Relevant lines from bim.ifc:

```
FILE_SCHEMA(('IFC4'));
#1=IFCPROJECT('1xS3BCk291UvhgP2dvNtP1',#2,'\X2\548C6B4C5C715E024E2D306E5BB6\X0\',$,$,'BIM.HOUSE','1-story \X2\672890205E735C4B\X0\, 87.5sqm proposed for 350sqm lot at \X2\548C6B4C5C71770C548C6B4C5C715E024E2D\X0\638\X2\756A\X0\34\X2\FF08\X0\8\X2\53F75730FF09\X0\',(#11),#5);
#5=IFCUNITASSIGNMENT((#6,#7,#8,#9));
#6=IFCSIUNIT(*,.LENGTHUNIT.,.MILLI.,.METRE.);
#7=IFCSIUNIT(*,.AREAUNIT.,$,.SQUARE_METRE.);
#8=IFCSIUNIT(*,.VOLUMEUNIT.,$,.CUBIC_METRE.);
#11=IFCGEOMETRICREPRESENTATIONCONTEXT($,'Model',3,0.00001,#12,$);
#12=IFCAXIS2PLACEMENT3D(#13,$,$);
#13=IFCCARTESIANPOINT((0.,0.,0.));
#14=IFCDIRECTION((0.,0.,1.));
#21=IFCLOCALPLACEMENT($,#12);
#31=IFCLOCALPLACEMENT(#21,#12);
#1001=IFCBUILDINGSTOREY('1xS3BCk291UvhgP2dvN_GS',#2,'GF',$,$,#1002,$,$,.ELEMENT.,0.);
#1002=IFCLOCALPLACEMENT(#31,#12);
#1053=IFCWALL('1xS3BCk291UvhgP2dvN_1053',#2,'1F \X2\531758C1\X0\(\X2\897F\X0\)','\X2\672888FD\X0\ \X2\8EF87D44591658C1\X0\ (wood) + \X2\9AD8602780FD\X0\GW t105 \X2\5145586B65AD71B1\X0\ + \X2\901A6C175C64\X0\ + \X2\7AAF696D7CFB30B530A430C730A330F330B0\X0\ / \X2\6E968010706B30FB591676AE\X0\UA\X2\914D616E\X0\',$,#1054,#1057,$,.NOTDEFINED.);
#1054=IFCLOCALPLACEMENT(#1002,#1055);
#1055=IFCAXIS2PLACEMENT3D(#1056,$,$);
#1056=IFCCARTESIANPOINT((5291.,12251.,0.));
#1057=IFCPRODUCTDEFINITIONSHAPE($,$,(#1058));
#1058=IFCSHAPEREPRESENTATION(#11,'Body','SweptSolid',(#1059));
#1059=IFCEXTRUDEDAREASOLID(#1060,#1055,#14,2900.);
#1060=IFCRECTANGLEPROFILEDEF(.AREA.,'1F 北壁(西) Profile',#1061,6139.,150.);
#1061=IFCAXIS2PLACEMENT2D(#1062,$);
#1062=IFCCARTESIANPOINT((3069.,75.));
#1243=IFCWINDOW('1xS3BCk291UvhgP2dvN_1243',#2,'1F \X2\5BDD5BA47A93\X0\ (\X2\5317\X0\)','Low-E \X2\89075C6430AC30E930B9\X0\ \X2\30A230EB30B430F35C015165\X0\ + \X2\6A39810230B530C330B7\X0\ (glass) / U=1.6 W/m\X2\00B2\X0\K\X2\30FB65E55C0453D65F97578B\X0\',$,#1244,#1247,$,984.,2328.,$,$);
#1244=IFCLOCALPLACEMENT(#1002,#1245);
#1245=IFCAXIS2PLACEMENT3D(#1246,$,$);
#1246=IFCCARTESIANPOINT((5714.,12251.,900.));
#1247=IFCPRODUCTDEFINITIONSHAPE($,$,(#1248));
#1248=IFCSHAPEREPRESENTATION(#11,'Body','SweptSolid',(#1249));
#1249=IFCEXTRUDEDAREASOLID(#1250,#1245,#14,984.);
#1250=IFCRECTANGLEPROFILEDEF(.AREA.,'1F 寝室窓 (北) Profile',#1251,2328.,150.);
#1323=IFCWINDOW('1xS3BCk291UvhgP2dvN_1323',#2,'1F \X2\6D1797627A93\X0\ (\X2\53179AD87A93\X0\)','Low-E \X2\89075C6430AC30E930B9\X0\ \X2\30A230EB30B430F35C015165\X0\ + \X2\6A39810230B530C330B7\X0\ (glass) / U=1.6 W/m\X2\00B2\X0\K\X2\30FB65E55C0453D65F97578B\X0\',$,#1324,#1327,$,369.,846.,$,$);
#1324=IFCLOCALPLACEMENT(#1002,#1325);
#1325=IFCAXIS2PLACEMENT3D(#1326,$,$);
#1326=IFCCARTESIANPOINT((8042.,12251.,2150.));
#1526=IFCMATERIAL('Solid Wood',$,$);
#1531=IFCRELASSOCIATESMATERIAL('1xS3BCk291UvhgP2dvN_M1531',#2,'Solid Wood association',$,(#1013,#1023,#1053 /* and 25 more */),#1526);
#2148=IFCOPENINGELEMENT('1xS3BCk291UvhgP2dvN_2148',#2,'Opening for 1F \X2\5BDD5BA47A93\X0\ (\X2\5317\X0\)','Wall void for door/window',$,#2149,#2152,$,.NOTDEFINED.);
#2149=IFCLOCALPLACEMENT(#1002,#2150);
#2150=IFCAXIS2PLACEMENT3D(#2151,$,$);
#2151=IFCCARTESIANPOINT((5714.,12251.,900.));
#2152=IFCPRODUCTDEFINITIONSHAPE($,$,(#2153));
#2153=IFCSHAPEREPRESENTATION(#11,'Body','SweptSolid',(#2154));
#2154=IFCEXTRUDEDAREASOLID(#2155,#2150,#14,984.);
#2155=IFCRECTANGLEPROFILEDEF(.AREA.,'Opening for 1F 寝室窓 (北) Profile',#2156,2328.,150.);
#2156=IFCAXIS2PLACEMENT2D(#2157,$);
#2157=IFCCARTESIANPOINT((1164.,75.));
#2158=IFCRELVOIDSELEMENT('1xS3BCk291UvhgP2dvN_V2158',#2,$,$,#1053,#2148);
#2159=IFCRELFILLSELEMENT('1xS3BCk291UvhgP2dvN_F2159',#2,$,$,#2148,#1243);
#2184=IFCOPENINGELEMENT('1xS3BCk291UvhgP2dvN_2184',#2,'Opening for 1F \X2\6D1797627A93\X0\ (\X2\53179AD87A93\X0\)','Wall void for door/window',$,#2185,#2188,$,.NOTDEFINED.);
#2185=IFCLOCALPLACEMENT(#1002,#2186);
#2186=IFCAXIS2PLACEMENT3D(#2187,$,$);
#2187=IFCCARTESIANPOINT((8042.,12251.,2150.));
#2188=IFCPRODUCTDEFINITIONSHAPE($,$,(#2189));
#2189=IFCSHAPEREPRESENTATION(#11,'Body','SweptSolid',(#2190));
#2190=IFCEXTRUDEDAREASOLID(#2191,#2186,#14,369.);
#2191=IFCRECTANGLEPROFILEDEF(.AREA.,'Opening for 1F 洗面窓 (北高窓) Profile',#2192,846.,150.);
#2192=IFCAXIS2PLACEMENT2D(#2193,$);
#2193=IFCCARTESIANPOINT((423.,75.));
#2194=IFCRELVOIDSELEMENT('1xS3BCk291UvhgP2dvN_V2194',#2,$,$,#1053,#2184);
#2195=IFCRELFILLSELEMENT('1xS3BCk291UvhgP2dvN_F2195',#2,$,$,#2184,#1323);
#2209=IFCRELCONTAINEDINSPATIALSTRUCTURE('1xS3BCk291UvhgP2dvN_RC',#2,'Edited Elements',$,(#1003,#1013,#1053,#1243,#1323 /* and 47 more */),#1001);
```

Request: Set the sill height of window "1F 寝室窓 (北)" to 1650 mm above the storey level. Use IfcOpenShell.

```python
import numpy as np
import ifcopenshell
import ifcopenshell.api.geometry
import ifcopenshell.geom
import ifcopenshell.util.element
import ifcopenshell.util.placement
import ifcopenshell.util.shape
import ifcopenshell.util.unit

model = ifcopenshell.open("bim.ifc")
unit_scale = ifcopenshell.util.unit.calculate_unit_scale(model)

window = model.by_guid("1xS3BCk291UvhgP2dvN_1243")
opening = window.FillsVoids[0].RelatingOpeningElement
storey = ifcopenshell.util.element.get_container(window, ifc_class="IfcBuildingStorey")
level = ifcopenshell.util.placement.get_local_placement(storey.ObjectPlacement)[2, 3]

# The opening's origin need not be at the sill, so measure its lowest point.
shape = ifcopenshell.geom.create_shape(ifcopenshell.geom.settings(), opening)
bottom = ifcopenshell.util.shape.get_shape_bottom_elevation(shape, shape.geometry) / unit_scale
dz = level + 1650.0 - bottom

shift = np.array([0.0, 0.0, dz])
# The window is not placed relative to its opening, so move both.
for product in (opening, window):
    matrix = ifcopenshell.util.placement.get_local_placement(product.ObjectPlacement)
    matrix[:3, 3] += shift
    ifcopenshell.api.geometry.edit_object_placement(model, product=product, matrix=matrix, is_si=False)

print(f"moved by {dz * unit_scale:+.3f} m")

model.write("bim_updated.ifc")
```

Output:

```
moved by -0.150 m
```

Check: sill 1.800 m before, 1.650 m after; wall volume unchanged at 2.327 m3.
